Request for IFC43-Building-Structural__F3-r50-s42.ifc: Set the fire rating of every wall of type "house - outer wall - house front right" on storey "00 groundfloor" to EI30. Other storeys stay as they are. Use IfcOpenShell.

First a look at what the model holds.

```python
import ifcopenshell
import ifcopenshell.util.element

model = ifcopenshell.open("IFC43-Building-Structural__F3-r50-s42.ifc")
print(model.schema)
storey = next(s for s in model.by_type("IfcBuildingStorey") if s.Name == "00 groundfloor")
walls = [e for e in ifcopenshell.util.element.get_decomposition(storey) if e.is_a("IfcWall")]
seen = {}
for e in walls:
    element_type = ifcopenshell.util.element.get_type(e)
    key = (element_type.Name if element_type != e and element_type else None, ifcopenshell.util.element.get_pset(e, "Pset_WallCommon", "FireRating"))
    seen[key] = seen.get(key, 0) + 1
for (name, value), count in sorted(seen.items(), key=str):
    print(count, "x", name, "|", value)
```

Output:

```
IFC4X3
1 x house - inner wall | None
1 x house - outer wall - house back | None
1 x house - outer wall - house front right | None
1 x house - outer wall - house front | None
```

```python
import ifcopenshell
import ifcopenshell.api.pset
import ifcopenshell.util.element

model = ifcopenshell.open("IFC43-Building-Structural__F3-r50-s42.ifc")

storey = next(s for s in model.by_type("IfcBuildingStorey") if s.Name == "00 groundfloor")
walls = [e for e in ifcopenshell.util.element.get_decomposition(storey) if e.is_a("IfcWall")]

count = 0
for e in walls:
    element_type = ifcopenshell.util.element.get_type(e)
    if element_type in (None, e) or element_type.Name != "house - outer wall - house front right":
        continue
    # add_pset returns the element's existing set when there is one.
    pset = ifcopenshell.api.pset.add_pset(model, product=e, name="Pset_WallCommon")
    ifcopenshell.api.pset.edit_pset(model, pset=pset, properties={"FireRating": "EI30"})
    count += 1

print(count, "walls updated")

model.write("IFC43-Building-Structural__F3-r50-s42-out.ifc")
```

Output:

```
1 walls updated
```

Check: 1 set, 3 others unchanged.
